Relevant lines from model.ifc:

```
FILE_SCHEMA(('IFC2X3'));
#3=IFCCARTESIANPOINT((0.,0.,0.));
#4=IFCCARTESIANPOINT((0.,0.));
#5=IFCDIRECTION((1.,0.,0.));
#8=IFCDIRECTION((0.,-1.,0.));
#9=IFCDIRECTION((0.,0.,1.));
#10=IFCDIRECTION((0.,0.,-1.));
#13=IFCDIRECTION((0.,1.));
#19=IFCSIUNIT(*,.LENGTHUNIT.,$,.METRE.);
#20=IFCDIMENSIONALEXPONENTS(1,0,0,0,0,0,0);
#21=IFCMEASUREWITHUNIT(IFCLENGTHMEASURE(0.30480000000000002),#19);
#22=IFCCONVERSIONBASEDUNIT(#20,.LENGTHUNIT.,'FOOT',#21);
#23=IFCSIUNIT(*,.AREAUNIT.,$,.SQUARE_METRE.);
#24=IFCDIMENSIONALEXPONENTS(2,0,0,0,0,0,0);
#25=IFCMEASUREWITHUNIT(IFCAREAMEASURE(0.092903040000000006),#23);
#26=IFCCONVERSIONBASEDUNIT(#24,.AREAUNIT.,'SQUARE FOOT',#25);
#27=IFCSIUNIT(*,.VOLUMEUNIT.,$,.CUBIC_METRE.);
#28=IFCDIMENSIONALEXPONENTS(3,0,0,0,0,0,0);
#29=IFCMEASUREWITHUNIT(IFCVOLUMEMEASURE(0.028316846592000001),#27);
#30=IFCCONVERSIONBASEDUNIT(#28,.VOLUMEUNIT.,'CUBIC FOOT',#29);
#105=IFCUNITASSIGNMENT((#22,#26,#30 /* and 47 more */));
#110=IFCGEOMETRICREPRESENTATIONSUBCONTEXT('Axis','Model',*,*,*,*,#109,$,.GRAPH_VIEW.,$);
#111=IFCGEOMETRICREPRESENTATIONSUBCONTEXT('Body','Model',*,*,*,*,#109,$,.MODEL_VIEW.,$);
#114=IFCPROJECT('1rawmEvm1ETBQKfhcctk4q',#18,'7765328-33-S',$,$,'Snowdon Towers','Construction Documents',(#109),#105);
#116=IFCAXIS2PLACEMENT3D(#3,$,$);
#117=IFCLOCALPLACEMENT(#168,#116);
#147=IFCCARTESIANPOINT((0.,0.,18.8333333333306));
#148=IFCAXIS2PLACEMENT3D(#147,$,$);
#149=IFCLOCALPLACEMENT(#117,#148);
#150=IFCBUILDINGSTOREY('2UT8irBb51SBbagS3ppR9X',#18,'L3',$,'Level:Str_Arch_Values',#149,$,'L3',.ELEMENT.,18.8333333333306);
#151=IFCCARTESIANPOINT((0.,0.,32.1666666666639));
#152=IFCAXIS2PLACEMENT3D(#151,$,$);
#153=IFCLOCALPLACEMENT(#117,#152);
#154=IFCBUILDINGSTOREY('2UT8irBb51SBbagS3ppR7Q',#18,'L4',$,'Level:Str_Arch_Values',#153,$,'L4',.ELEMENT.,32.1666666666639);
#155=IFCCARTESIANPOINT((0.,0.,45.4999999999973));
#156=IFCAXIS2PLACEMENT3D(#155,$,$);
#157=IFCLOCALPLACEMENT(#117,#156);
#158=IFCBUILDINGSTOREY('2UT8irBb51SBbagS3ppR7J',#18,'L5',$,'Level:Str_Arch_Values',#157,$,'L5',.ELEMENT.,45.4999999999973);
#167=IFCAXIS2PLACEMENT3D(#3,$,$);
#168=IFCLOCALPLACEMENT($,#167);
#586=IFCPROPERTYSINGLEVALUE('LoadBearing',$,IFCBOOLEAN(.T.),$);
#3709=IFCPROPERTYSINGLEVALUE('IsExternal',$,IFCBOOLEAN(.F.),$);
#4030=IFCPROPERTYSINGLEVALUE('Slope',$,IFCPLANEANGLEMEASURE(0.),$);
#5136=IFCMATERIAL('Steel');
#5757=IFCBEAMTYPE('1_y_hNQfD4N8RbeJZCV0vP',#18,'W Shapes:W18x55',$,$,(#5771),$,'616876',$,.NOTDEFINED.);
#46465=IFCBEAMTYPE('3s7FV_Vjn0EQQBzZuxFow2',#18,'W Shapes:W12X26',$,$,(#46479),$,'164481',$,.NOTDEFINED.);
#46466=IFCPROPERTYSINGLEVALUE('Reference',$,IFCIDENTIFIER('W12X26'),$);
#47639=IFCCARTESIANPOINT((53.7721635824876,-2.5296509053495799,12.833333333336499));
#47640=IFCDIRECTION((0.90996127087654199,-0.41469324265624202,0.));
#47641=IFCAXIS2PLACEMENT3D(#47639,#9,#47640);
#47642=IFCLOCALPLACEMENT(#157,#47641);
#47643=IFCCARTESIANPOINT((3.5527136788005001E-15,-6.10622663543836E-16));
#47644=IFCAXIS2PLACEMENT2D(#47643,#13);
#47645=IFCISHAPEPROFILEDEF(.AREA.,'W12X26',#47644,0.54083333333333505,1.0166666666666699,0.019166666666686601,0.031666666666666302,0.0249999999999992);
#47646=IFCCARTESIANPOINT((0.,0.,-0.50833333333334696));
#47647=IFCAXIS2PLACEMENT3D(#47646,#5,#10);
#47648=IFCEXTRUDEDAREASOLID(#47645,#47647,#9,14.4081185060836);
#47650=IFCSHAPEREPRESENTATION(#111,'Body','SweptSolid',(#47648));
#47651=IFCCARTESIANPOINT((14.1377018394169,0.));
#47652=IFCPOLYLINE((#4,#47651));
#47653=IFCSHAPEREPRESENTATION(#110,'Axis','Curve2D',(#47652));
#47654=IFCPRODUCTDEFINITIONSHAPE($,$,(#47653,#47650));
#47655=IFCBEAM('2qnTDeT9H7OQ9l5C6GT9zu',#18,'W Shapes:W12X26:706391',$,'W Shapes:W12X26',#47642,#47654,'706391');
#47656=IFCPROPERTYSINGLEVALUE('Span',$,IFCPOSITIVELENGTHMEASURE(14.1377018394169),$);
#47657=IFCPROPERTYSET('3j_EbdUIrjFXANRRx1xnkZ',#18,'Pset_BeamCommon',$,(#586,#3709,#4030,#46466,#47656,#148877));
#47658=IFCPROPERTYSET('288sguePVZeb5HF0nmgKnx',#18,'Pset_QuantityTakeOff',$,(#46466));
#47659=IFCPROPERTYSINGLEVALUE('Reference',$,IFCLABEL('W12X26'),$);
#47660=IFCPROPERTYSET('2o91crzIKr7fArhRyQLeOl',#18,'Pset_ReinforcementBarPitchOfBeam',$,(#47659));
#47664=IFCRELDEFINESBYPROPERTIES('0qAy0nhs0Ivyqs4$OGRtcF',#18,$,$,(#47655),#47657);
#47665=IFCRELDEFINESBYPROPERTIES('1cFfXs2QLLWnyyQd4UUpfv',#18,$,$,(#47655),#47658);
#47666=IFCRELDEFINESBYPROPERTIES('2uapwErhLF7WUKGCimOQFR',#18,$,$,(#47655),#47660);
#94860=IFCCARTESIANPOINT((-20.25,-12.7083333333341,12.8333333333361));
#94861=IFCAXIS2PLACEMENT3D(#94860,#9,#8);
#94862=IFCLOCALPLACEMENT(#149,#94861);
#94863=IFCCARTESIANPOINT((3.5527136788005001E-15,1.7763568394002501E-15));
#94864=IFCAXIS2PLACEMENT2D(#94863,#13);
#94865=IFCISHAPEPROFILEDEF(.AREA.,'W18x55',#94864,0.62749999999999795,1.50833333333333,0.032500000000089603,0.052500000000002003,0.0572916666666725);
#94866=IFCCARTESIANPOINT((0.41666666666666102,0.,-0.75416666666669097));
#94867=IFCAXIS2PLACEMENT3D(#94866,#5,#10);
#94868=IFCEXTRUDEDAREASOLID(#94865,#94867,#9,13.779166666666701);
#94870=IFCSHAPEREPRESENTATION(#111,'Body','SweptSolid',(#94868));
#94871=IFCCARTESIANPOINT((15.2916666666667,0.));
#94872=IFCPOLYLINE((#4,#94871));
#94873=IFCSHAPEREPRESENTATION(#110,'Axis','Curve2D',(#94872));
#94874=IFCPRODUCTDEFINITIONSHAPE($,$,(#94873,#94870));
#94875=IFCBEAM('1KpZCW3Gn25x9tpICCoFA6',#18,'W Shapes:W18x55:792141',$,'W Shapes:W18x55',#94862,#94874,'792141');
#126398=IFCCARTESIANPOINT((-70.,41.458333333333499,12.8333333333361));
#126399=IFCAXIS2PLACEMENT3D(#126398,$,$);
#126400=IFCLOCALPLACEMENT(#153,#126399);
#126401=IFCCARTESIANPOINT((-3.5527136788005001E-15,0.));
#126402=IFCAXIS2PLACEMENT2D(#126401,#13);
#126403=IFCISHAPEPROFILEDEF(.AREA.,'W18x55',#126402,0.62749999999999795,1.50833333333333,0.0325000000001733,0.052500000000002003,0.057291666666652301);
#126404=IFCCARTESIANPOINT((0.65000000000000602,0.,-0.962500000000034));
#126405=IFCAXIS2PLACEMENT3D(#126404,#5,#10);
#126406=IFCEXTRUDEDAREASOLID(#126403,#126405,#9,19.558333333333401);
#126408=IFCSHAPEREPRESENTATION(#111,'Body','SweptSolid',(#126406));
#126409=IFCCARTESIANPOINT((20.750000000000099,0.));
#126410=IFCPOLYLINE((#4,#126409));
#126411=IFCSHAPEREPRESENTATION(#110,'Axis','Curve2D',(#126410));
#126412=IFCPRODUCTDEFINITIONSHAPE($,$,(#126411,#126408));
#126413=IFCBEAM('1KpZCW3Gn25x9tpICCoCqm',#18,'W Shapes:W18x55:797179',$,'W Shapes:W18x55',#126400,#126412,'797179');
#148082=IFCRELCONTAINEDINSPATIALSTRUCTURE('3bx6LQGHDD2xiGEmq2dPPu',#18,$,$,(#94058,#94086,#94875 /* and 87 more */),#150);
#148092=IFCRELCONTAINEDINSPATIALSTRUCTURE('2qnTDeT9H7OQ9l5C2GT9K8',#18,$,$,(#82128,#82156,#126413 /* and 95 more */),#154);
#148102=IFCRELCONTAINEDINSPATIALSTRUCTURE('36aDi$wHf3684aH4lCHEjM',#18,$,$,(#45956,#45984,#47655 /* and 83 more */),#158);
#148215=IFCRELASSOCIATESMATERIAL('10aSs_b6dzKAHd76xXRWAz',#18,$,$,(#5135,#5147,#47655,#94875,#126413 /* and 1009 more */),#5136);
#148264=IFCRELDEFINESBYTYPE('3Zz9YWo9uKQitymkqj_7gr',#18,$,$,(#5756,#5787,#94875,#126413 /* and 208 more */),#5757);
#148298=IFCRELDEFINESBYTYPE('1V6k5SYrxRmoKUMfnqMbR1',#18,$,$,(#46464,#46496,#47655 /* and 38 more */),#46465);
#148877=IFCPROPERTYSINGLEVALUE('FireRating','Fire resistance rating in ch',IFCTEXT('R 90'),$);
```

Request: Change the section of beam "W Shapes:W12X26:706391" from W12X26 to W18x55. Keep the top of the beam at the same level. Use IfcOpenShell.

```python
import ifcopenshell
import ifcopenshell.api.pset
import ifcopenshell.api.type
import ifcopenshell.util.element
import ifcopenshell.util.representation

model = ifcopenshell.open("model.ifc")

member = model.by_guid("2qnTDeT9H7OQ9l5C6GT9zu")
source = next(p for p in model.by_type("IfcIShapeProfileDef") if p.ProfileName == "W18x55")

body = ifcopenshell.util.representation.get_representation(member, "Model", "Body")
solid = body.Items[0]
old_profile = solid.SweptArea

# Copy the section's sizes but keep this member's own profile position.
profile = ifcopenshell.util.element.copy(model, source)
# Profiles are centred, so shift by half the change in depth to hold the top.
shift = (old_profile.OverallDepth - profile.OverallDepth) / 2
x, y = old_profile.Position.Location.Coordinates
up = (-1.0, 0.0)  # upwards, in the solid's own plane
location = model.createIfcCartesianPoint((x + up[0] * shift, y + up[1] * shift))
profile.Position = model.createIfcAxis2Placement2D(location, old_profile.Position.RefDirection)
solid.SweptArea = profile
if not model.get_total_inverses(old_profile):
    ifcopenshell.util.element.remove_deep2(model, old_profile)

new_type = model.by_guid("1_y_hNQfD4N8RbeJZCV0vP")
ifcopenshell.api.type.assign_type(
    model, related_objects=[member], relating_type=new_type, should_map_representations=False
)
member.Name = member.Name.replace("W12X26", "W18x55")
member.ObjectType = "W Shapes:W18x55"
pset = model.by_id(ifcopenshell.util.element.get_pset(member, "Pset_BeamCommon", should_inherit=False)["id"])
ifcopenshell.api.pset.edit_pset(model, pset=pset, properties={"Reference": "W18x55"})
pset = model.by_id(ifcopenshell.util.element.get_pset(member, "Pset_QuantityTakeOff", should_inherit=False)["id"])
ifcopenshell.api.pset.edit_pset(model, pset=pset, properties={"Reference": "W18x55"})
pset = model.by_id(ifcopenshell.util.element.get_pset(member, "Pset_ReinforcementBarPitchOfBeam", should_inherit=False)["id"])
ifcopenshell.api.pset.edit_pset(model, pset=pset, properties={"Reference": "W18x55"})

print(solid.SweptArea)

model.write("model_v2.ifc")
```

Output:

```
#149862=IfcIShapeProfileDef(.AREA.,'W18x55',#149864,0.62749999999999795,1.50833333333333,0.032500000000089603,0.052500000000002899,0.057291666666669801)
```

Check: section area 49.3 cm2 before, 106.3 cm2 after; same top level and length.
